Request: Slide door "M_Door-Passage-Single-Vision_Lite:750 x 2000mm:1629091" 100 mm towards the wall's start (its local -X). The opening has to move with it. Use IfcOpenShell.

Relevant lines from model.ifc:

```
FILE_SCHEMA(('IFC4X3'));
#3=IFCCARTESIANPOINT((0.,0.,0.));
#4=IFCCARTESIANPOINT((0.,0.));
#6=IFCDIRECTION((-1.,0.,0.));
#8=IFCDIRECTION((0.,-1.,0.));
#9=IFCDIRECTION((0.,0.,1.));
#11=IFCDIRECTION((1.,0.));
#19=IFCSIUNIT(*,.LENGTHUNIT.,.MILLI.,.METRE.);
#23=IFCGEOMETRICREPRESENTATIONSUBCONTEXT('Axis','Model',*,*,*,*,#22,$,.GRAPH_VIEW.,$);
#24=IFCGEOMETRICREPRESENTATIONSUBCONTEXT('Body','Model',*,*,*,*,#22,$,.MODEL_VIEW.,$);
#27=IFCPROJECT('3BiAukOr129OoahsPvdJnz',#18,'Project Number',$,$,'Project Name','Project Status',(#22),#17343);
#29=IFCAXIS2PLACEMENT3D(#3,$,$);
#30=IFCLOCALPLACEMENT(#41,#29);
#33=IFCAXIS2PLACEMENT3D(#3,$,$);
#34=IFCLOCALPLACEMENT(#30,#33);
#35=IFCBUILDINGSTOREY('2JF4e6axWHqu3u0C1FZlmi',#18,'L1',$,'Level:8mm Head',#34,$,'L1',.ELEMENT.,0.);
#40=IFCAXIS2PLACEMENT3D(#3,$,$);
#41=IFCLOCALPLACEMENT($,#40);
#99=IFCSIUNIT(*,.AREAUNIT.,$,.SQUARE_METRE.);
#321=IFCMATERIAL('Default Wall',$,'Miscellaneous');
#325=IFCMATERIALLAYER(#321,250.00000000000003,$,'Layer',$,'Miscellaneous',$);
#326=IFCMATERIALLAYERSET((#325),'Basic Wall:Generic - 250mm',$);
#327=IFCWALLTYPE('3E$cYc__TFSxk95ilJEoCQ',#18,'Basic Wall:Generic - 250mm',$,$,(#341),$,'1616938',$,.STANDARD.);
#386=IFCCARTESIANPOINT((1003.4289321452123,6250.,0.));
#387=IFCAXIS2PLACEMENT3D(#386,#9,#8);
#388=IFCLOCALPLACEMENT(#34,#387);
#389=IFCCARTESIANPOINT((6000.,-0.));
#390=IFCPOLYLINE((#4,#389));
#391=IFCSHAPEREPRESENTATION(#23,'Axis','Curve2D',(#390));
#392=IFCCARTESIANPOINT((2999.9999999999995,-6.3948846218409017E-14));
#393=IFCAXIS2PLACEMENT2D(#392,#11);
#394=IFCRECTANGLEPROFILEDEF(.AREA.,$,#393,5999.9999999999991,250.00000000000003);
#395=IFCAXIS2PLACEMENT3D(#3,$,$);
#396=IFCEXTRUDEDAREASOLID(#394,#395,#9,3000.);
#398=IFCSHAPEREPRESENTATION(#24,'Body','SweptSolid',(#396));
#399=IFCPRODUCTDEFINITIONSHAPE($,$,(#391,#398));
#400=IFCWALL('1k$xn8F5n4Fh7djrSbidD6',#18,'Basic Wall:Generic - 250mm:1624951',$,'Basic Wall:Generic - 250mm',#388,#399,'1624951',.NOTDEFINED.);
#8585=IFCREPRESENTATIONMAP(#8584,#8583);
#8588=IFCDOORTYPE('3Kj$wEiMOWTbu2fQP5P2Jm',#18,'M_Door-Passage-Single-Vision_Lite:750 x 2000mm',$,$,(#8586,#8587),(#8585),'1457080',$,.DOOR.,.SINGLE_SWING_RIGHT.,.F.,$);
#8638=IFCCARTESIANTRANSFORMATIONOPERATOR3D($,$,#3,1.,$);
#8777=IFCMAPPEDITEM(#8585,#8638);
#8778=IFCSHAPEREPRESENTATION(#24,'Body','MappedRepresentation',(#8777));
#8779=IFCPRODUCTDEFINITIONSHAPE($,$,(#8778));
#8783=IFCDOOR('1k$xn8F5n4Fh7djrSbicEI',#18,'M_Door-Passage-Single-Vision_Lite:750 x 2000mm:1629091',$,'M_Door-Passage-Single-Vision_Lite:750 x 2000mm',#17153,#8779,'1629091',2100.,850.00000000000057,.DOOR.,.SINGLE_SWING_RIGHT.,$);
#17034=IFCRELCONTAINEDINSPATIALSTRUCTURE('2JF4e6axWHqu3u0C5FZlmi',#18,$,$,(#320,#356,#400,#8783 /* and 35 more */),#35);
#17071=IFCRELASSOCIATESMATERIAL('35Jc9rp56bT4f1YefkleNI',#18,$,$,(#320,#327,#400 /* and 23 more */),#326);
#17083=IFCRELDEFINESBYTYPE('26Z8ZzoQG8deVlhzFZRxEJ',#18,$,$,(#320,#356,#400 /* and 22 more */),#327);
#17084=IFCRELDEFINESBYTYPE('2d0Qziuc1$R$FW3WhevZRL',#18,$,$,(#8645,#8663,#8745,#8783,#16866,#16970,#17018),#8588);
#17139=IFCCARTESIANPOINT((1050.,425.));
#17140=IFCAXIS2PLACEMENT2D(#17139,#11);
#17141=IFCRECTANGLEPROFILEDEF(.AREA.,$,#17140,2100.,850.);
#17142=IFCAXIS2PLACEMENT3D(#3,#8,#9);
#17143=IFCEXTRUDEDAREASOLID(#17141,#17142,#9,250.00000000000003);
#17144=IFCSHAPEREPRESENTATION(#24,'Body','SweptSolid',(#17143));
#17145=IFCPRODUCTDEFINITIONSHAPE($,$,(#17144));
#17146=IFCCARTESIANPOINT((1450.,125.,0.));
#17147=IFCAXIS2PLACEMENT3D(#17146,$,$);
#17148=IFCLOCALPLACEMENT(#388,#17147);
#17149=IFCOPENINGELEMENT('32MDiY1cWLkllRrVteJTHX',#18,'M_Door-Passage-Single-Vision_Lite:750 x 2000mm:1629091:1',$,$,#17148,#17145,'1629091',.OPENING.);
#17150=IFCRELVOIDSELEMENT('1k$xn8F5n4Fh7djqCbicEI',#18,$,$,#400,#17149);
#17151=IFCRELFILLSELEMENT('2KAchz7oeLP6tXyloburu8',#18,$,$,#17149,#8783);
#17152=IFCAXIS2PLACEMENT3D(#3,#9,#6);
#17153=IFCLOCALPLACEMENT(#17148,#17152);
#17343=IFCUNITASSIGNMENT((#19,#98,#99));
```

```python
import ifcopenshell
import ifcopenshell.api.geometry
import ifcopenshell.util.placement
import ifcopenshell.util.unit

model = ifcopenshell.open("model.ifc")
unit_scale = ifcopenshell.util.unit.calculate_unit_scale(model)

door = model.by_id(8783)
opening = door.FillsVoids[0].RelatingOpeningElement
wall = opening.VoidsElements[0].RelatingBuildingElement

wall_matrix = ifcopenshell.util.placement.get_local_placement(wall.ObjectPlacement)
shift = wall_matrix[:3, 0] * -0.1 / unit_scale
before = ifcopenshell.util.placement.get_local_placement(door.ObjectPlacement)[:3, 3].copy()

# The door is placed relative to its opening, so it follows when the opening moves.
matrix = ifcopenshell.util.placement.get_local_placement(opening.ObjectPlacement)
matrix[:3, 3] += shift
ifcopenshell.api.geometry.edit_object_placement(
    model, product=opening, matrix=matrix, is_si=False, should_transform_children=True
)

after = ifcopenshell.util.placement.get_local_placement(door.ObjectPlacement)[:3, 3]
print("door moved by", (after - before).round(3) + 0.0)

model.write("model_rev.ifc")
```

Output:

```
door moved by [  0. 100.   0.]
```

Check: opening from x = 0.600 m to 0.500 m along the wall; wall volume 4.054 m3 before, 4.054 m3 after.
